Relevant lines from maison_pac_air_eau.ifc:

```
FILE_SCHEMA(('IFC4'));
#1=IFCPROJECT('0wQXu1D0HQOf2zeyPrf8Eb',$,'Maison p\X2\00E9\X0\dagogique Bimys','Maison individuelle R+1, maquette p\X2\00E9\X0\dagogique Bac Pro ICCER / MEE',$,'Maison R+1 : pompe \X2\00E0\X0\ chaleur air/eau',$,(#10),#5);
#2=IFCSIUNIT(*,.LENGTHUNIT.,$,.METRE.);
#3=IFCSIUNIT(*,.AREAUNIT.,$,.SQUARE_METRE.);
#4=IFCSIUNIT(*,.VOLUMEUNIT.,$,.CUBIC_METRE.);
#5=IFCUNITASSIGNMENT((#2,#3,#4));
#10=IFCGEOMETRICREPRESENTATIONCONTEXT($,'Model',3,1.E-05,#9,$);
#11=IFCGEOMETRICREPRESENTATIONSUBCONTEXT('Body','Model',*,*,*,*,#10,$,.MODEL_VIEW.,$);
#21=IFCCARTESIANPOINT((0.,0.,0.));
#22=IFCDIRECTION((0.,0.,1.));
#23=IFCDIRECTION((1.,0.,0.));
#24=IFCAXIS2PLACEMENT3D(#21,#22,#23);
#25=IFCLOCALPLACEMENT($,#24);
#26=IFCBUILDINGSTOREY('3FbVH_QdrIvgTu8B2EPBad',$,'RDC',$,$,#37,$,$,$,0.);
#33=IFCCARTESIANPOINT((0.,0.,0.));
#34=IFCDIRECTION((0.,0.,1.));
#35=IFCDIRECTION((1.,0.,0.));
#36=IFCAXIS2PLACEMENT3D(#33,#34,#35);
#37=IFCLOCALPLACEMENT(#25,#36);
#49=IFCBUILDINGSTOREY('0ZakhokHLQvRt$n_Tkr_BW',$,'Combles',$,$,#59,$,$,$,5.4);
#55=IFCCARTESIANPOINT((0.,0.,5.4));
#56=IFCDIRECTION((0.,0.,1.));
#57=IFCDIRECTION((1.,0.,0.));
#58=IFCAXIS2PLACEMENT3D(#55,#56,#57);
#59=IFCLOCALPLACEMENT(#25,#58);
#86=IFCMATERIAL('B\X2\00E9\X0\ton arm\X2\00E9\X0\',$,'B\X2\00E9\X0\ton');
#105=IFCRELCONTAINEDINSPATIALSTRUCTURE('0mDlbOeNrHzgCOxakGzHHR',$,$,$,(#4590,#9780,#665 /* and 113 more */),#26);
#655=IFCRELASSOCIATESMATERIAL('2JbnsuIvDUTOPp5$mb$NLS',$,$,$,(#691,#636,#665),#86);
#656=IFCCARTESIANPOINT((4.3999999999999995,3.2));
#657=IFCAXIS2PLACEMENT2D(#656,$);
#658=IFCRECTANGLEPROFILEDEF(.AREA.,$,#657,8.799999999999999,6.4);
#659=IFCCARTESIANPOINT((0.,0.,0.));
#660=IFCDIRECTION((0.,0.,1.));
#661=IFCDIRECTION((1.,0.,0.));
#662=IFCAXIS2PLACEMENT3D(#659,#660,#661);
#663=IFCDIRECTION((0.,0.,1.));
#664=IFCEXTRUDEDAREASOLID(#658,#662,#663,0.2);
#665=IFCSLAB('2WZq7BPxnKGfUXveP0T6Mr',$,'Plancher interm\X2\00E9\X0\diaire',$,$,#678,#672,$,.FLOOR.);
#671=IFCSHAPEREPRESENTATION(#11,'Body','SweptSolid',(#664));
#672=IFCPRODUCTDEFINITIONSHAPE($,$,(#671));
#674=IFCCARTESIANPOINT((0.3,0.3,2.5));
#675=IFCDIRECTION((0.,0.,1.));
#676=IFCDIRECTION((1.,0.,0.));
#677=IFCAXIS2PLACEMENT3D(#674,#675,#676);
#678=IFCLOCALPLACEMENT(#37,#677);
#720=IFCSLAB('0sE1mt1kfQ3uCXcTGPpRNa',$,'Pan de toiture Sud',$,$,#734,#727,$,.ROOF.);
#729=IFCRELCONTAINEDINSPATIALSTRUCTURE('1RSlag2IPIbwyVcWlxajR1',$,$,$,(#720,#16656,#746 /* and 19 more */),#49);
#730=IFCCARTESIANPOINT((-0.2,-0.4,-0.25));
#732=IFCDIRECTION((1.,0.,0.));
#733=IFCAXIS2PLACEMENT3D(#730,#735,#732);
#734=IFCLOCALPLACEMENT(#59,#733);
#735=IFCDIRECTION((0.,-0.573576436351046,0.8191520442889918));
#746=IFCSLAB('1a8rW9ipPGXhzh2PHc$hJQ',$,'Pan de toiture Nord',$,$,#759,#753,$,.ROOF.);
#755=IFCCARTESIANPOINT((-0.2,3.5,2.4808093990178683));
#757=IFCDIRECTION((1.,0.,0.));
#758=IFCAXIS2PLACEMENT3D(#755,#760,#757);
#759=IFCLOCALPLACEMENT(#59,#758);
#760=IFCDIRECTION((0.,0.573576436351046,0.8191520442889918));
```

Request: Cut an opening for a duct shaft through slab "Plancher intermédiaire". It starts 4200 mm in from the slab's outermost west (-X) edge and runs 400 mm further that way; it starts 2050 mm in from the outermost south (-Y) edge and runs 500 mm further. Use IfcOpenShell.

```python
import numpy as np
import ifcopenshell
import ifcopenshell.api.feature
import ifcopenshell.api.geometry
import ifcopenshell.api.root
import ifcopenshell.geom
import ifcopenshell.util.placement
import ifcopenshell.util.representation
import ifcopenshell.util.shape
import ifcopenshell.util.unit

model = ifcopenshell.open("maison_pac_air_eau.ifc")
unit_scale = ifcopenshell.util.unit.calculate_unit_scale(model)
settings = ifcopenshell.geom.settings()


def volume(element):
    """Net volume in cubic metres, openings subtracted."""
    shape = ifcopenshell.geom.create_shape(settings, element)
    return ifcopenshell.util.shape.get_volume(shape.geometry)


slab = model.by_guid("2WZq7BPxnKGfUXveP0T6Mr")
before = volume(slab)

# Extent in the slab's own axes, in metres. The edges named are its -X and -Y sides.
slab_shape = ifcopenshell.geom.create_shape(settings, slab)
vertices = ifcopenshell.util.shape.get_vertices(slab_shape.geometry)
x_min, y_min, bottom = vertices.min(axis=0)
top = vertices[:, 2].max()

opening = ifcopenshell.api.root.create_entity(model, ifc_class="IfcOpeningElement", name="Duct shaft opening", predefined_type="OPENING")
context = ifcopenshell.util.representation.get_context(model, "Model", "Body", "MODEL_VIEW")
width, depth = 0.4, 0.5
outline = [(0.0, 0.0), (width, 0.0), (width, depth), (0.0, depth), (0.0, 0.0)]
# Overshoot both faces by 50 mm so the cut is clean.
shape = ifcopenshell.api.geometry.add_slab_representation(
    model, context=context, depth=top - bottom + 0.1, polyline=outline
)
ifcopenshell.api.geometry.assign_representation(model, product=opening, representation=shape)

matrix = ifcopenshell.util.placement.get_local_placement(slab.ObjectPlacement)
matrix[:, 3] = matrix @ np.append(np.array([x_min + 4.2, y_min + 2.05, bottom - 0.05]) / unit_scale, 1.0)
ifcopenshell.api.geometry.edit_object_placement(model, product=opening, matrix=matrix, is_si=False)
ifcopenshell.api.feature.add_feature(model, feature=opening, element=slab)

after = volume(slab)

print(f"slab volume {before:.3f} -> {after:.3f} m3")

model.write("maison_pac_air_eau_updated.ifc")
```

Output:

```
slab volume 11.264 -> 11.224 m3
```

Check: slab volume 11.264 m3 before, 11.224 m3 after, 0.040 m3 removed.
